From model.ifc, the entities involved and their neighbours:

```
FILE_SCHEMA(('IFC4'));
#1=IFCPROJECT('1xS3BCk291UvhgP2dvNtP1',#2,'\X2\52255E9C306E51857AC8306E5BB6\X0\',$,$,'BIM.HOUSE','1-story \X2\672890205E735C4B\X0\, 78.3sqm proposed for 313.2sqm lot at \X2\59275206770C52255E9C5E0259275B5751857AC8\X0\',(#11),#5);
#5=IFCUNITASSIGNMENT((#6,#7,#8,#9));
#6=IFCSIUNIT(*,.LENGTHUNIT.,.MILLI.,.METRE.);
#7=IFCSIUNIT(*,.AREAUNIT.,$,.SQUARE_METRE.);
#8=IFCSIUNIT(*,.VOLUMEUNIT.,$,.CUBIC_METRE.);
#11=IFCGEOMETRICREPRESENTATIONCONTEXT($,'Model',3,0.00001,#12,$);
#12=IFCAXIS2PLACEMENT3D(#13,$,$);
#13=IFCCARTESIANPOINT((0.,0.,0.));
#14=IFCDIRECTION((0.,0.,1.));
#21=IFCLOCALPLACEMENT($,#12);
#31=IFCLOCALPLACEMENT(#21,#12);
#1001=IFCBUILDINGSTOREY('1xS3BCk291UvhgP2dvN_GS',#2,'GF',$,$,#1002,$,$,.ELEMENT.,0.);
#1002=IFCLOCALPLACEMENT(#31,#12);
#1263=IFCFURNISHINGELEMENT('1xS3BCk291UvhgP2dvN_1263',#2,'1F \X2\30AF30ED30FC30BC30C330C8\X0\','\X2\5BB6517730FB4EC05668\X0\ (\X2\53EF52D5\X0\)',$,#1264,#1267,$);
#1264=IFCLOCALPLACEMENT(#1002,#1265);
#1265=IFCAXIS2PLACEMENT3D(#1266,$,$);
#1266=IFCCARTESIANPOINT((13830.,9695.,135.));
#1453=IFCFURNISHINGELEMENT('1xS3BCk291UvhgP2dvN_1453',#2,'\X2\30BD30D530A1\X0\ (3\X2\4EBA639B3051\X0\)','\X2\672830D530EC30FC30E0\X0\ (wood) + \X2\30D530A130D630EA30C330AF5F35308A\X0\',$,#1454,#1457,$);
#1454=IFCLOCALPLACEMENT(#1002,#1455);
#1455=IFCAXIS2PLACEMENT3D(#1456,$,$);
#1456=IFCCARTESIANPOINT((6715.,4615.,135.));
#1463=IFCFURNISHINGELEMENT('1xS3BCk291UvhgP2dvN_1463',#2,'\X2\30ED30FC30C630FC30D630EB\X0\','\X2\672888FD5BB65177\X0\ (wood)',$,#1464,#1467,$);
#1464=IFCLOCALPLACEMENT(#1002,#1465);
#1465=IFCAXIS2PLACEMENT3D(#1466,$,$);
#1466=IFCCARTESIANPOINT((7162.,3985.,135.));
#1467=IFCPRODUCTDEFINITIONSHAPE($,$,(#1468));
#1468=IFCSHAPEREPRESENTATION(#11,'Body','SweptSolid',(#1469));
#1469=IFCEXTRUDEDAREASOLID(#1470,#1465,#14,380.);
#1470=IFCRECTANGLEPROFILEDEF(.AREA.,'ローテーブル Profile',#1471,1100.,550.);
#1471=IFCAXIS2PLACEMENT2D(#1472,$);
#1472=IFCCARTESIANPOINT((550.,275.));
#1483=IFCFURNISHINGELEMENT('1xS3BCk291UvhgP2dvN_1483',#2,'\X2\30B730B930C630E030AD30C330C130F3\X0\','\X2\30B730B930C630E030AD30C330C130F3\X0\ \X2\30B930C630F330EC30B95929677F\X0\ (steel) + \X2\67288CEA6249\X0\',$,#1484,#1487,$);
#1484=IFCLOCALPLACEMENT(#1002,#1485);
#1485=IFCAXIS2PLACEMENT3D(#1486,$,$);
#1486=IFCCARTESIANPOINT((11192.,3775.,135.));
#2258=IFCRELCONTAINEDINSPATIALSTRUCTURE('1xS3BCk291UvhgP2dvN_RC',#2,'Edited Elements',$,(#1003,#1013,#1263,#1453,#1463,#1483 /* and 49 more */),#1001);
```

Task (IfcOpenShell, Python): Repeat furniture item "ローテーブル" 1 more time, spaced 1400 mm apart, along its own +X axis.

```python
import ifcopenshell
import ifcopenshell.api.geometry
import ifcopenshell.api.root
import ifcopenshell.util.element
import ifcopenshell.util.placement
import ifcopenshell.util.unit

model = ifcopenshell.open("model.ifc")
unit_scale = ifcopenshell.util.unit.calculate_unit_scale(model)


def reuse_history(source, copy):
    """copy_class also copies each property set's owner history, people and application; keep the originals."""
    for rel in copy.IsDefinedBy:
        if rel.is_a("IfcRelDefinesByProperties") and (history := rel.RelatingPropertyDefinition.OwnerHistory):
            rel.RelatingPropertyDefinition.OwnerHistory = source.OwnerHistory
            ifcopenshell.util.element.remove_deep2(model, history)


source = model.by_id(1463)
base = ifcopenshell.util.placement.get_local_placement(source.ObjectPlacement)
step = base[:3, 0] * 1.4 / unit_scale

for i in range(1, 2):
    copy = ifcopenshell.api.root.copy_class(model, product=source)
    copy.Representation = ifcopenshell.util.element.copy_deep(
        model, source.Representation, exclude=["IfcGeometricRepresentationContext", "IfcRepresentationMap"]
    )
    reuse_history(source, copy)
    matrix = base.copy()
    matrix[:3, 3] += i * step
    print("added at", matrix[:3, 3].round(3) + 0.0)
    ifcopenshell.api.geometry.edit_object_placement(model, product=copy, matrix=matrix, is_si=False)

model.write("model_updated.ifc")
```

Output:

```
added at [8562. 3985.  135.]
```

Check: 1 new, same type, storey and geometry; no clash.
